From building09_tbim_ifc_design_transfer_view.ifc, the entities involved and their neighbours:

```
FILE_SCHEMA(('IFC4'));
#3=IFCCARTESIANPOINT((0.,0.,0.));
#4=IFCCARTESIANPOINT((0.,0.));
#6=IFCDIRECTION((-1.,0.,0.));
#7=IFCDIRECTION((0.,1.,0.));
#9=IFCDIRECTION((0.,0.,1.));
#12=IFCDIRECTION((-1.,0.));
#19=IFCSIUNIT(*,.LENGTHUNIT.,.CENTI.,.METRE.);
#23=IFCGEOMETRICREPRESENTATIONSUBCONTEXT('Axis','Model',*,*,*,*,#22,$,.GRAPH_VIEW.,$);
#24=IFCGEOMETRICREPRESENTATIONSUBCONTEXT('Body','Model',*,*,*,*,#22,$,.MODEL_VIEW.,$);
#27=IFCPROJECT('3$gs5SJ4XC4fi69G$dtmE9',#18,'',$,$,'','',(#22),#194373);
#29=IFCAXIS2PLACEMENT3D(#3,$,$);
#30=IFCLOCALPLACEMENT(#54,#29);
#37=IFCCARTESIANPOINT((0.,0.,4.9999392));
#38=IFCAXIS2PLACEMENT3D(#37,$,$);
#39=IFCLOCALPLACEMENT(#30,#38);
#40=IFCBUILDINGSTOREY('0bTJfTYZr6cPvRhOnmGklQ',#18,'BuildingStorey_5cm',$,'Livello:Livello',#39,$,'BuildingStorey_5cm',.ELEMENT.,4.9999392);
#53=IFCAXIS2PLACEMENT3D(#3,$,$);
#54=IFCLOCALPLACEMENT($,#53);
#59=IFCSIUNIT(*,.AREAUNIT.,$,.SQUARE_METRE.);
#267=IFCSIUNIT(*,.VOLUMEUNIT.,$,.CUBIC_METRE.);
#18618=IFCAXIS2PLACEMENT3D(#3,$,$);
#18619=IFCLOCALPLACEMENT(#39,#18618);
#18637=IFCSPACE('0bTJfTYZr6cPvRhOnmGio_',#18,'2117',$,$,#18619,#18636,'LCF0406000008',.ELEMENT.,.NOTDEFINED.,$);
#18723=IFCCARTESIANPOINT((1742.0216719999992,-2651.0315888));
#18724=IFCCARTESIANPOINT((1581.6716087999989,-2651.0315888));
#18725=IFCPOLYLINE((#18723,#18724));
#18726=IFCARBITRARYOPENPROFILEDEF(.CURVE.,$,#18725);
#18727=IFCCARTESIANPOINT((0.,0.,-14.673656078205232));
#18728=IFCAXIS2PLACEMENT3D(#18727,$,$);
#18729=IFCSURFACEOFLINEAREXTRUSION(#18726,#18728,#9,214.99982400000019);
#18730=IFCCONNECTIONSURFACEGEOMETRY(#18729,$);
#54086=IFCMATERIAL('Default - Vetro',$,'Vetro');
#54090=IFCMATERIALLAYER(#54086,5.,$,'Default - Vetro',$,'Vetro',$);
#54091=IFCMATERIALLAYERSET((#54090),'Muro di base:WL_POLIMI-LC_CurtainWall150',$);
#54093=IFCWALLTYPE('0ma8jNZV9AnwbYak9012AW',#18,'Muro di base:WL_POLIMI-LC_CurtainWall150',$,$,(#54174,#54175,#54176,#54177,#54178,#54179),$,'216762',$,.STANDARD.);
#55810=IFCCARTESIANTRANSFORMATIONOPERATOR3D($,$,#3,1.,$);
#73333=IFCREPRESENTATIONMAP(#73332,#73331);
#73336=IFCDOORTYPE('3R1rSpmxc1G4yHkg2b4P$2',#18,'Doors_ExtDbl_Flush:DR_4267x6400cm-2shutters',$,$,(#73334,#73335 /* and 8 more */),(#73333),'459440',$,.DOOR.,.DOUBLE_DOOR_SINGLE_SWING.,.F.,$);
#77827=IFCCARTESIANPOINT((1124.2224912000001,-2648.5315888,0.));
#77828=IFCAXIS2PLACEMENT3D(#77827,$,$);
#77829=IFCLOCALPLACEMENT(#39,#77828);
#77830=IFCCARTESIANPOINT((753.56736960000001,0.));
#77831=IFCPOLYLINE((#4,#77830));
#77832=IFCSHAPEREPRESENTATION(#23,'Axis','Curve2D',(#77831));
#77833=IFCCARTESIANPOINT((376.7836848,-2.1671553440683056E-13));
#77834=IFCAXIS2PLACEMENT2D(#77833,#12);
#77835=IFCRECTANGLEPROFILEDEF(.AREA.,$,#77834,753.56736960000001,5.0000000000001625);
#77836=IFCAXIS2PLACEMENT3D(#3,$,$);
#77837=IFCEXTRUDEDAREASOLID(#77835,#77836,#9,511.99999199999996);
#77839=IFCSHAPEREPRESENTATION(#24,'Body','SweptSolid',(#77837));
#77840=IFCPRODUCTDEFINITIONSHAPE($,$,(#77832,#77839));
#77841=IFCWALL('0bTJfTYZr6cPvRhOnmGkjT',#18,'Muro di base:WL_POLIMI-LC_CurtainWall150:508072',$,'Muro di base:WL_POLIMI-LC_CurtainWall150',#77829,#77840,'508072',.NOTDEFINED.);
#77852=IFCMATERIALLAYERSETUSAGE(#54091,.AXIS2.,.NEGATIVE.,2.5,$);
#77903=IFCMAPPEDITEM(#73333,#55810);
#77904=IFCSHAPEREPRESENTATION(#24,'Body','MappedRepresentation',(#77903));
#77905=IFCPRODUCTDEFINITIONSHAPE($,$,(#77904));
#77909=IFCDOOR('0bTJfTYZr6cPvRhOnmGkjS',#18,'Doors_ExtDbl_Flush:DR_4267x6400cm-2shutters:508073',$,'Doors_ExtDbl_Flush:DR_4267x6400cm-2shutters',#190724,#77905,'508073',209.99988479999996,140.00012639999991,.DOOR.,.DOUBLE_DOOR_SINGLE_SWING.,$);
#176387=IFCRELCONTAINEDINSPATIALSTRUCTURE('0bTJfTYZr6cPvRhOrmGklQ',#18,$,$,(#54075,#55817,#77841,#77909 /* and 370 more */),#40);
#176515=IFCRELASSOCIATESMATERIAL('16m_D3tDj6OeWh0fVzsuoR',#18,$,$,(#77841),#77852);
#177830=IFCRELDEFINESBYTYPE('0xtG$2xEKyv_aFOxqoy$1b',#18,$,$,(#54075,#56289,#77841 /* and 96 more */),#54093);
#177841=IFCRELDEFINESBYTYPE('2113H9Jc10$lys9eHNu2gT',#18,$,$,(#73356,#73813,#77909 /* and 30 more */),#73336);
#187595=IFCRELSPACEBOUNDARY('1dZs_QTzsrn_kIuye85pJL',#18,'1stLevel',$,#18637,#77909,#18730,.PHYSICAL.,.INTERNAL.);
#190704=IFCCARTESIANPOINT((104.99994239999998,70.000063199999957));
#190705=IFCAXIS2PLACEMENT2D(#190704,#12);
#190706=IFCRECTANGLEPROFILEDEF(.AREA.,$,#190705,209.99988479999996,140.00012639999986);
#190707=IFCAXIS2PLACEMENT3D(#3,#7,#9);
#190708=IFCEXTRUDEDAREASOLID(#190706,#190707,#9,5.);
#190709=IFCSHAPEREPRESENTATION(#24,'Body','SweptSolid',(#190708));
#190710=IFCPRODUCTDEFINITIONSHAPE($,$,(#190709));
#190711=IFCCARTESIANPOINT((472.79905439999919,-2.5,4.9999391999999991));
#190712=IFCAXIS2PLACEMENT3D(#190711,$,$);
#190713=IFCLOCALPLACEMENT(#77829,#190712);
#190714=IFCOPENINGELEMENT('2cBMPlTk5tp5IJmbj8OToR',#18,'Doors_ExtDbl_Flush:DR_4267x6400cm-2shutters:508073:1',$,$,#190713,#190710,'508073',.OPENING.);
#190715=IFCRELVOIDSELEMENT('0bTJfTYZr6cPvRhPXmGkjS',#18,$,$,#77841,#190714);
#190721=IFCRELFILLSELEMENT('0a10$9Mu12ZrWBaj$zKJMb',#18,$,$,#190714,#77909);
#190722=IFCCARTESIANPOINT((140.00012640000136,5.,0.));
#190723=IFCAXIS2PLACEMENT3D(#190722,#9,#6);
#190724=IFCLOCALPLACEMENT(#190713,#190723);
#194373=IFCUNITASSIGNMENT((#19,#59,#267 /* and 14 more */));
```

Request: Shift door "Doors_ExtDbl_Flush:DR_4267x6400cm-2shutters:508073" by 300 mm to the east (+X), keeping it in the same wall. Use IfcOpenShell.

```python
import numpy as np
import ifcopenshell
import ifcopenshell.api.geometry
import ifcopenshell.util.placement
import ifcopenshell.util.unit

model = ifcopenshell.open("building09_tbim_ifc_design_transfer_view.ifc")
unit_scale = ifcopenshell.util.unit.calculate_unit_scale(model)

door = model.by_id(77909)
opening = door.FillsVoids[0].RelatingOpeningElement
wall = opening.VoidsElements[0].RelatingBuildingElement

wall_matrix = ifcopenshell.util.placement.get_local_placement(wall.ObjectPlacement)
shift = wall_matrix[:3, 0] * 0.3 / unit_scale
before = ifcopenshell.util.placement.get_local_placement(door.ObjectPlacement)[:3, 3].copy()

# The door is placed relative to its opening, so it follows when the opening moves.
matrix = ifcopenshell.util.placement.get_local_placement(opening.ObjectPlacement)
matrix[:3, 3] += shift
ifcopenshell.api.geometry.edit_object_placement(
    model, product=opening, matrix=matrix, is_si=False, should_transform_children=True
)

# Space boundary surfaces are stored in each space's coordinates; move them too.
for rel in door.ProvidesBoundaries:
    if not rel.ConnectionGeometry:
        continue
    surface = rel.ConnectionGeometry.SurfaceOnRelatingElement
    space_matrix = ifcopenshell.util.placement.get_local_placement(rel.RelatingSpace.ObjectPlacement)
    point = np.array(surface.Position.Location.Coordinates) + space_matrix[:3, :3].T @ shift
    surface.Position = model.createIfcAxis2Placement3D(
        model.createIfcCartesianPoint(point.tolist()), surface.Position.Axis, surface.Position.RefDirection
    )

after = ifcopenshell.util.placement.get_local_placement(door.ObjectPlacement)[:3, 3]
print("door moved by", (after - before).round(3) + 0.0)

model.write("building09_tbim_ifc_design_transfer_view_v2.ifc")
```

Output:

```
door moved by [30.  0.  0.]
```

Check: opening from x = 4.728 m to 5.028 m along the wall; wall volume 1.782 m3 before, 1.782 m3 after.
